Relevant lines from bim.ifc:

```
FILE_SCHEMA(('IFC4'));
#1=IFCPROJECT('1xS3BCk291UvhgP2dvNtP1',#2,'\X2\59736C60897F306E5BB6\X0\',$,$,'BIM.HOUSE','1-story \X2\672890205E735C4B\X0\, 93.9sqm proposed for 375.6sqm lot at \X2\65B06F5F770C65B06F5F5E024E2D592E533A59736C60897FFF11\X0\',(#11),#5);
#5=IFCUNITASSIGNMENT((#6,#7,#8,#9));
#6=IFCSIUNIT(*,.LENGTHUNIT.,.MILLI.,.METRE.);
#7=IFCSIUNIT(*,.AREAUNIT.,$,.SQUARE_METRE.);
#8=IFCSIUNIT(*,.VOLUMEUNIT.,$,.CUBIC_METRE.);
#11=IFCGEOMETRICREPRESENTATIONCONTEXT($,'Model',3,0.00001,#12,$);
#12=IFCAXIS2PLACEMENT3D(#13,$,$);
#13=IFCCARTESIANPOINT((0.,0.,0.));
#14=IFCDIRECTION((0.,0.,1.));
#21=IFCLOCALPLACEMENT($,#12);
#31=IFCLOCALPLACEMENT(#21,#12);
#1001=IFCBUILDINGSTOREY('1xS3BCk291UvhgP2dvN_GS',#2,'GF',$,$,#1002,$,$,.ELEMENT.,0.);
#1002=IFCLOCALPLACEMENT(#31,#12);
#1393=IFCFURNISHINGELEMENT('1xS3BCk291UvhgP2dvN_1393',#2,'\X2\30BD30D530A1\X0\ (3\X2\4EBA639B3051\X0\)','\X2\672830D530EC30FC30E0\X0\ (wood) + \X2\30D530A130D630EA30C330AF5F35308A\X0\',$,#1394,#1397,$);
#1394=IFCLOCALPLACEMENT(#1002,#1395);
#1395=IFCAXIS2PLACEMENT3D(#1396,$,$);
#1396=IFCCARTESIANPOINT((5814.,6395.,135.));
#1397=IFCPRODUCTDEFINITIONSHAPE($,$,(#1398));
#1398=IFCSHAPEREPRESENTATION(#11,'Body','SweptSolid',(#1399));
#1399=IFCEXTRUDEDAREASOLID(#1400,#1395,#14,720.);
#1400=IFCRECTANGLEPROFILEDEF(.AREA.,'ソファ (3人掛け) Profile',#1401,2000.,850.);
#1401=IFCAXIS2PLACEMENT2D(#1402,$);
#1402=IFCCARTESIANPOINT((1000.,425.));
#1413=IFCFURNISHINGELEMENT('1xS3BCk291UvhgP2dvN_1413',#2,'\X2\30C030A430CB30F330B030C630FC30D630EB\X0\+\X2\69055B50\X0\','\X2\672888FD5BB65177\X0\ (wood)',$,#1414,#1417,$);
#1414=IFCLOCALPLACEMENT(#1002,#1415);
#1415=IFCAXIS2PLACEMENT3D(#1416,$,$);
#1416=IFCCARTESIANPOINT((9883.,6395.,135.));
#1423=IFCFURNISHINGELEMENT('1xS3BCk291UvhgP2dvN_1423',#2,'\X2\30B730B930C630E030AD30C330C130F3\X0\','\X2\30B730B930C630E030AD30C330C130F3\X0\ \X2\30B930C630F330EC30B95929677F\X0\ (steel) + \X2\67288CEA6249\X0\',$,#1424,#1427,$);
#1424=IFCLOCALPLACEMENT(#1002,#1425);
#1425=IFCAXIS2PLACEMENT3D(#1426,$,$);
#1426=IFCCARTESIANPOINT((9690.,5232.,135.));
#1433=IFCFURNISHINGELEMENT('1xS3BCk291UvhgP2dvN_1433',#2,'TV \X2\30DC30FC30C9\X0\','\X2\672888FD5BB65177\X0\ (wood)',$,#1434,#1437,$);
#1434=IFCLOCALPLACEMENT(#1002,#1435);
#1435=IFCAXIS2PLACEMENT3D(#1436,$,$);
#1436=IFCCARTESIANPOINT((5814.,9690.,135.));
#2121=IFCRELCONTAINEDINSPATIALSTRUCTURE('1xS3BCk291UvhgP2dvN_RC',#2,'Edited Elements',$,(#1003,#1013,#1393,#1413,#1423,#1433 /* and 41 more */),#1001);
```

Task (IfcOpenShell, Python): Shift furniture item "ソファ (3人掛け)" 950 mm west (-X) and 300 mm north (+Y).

```python
import ifcopenshell
import ifcopenshell.api.geometry
import ifcopenshell.util.placement
import ifcopenshell.util.unit

model = ifcopenshell.open("bim.ifc")
unit_scale = ifcopenshell.util.unit.calculate_unit_scale(model)

item = model.by_guid("1xS3BCk291UvhgP2dvN_1393")
matrix = ifcopenshell.util.placement.get_local_placement(item.ObjectPlacement)
matrix[0, 3] -= 0.95 / unit_scale
matrix[1, 3] += 0.3 / unit_scale
ifcopenshell.api.geometry.edit_object_placement(model, product=item, matrix=matrix, is_si=False)

print(ifcopenshell.util.placement.get_local_placement(item.ObjectPlacement).round(3) + 0.0)

model.write("bim_v2.ifc")
```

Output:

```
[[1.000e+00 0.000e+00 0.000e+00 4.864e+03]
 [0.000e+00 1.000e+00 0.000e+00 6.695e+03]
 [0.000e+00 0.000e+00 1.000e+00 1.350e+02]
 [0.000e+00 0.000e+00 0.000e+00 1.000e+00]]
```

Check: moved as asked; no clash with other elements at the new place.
